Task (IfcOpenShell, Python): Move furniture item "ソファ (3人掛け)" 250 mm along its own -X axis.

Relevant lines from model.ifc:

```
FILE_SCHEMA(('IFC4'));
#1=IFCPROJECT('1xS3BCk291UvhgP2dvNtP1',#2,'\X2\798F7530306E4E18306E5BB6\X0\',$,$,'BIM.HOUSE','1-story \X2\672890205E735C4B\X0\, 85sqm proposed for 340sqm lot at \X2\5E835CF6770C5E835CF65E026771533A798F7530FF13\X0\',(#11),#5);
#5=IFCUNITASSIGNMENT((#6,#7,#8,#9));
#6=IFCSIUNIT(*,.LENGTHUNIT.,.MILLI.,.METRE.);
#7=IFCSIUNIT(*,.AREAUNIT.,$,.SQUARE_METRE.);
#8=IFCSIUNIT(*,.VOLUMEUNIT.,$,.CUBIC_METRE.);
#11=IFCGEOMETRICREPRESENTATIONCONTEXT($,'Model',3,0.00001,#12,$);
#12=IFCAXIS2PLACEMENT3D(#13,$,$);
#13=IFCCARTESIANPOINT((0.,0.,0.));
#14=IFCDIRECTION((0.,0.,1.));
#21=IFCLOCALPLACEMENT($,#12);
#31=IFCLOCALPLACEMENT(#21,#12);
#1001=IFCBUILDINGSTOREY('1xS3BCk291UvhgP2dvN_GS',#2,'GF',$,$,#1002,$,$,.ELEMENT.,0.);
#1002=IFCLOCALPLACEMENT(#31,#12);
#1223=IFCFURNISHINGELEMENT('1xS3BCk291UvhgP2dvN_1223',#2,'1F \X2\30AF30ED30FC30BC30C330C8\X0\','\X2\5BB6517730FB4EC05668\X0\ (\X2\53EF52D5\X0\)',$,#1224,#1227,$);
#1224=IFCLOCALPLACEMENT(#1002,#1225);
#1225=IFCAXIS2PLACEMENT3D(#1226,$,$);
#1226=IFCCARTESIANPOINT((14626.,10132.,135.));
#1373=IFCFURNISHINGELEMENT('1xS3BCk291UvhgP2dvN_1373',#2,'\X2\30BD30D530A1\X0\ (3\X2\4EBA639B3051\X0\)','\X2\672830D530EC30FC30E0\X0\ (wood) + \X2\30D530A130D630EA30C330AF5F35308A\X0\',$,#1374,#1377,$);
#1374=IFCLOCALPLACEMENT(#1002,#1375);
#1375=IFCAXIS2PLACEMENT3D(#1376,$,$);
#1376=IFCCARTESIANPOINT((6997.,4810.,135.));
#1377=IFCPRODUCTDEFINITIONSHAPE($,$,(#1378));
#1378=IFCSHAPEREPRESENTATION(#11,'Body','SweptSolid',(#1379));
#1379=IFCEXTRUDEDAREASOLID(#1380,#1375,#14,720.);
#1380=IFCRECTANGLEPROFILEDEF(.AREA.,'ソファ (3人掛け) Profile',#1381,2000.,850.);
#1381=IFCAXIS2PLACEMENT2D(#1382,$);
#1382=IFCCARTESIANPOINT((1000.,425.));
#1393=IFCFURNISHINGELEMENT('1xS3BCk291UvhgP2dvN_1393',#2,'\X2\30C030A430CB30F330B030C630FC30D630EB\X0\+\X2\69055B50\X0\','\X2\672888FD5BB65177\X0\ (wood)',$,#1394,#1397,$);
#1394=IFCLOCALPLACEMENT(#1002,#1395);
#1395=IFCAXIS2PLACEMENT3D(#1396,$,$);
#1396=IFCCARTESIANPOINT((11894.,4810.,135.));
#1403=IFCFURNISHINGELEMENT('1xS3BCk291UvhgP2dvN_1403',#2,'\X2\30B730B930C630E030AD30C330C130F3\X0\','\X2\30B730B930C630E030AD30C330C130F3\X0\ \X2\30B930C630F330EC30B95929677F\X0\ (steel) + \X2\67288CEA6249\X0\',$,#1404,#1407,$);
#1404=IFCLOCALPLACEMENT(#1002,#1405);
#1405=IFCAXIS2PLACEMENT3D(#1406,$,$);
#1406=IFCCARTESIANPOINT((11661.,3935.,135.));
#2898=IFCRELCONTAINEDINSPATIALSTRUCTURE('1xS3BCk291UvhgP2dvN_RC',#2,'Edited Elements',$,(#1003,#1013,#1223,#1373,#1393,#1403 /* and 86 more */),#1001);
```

```python
import ifcopenshell
import ifcopenshell.api.geometry
import ifcopenshell.util.placement

model = ifcopenshell.open("model.ifc")

item = model.by_id(1373)
matrix = ifcopenshell.util.placement.get_local_placement(item.ObjectPlacement)
matrix[:3, 3] -= matrix[:3, 0] * 250.0
ifcopenshell.api.geometry.edit_object_placement(model, product=item, matrix=matrix, is_si=False)

print(ifcopenshell.util.placement.get_local_placement(item.ObjectPlacement).round(3) + 0.0)

model.write("model_v2.ifc")
```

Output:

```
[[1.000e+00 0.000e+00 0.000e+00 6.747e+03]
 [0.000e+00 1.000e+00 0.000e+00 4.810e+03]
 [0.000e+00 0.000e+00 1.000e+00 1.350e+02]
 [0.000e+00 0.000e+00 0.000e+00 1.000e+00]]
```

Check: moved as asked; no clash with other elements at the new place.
